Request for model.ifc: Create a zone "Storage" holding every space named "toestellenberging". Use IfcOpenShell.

First a look at what the model holds.

```python
import ifcopenshell

model = ifcopenshell.open("model.ifc")
print(model.schema)
seen = {}
for space in model.by_type("IfcSpace"):
    seen[space.LongName] = seen.get(space.LongName, 0) + 1
for name, count in sorted(seen.items(), key=str):
    print(count, "x", name)
print("zones:", [z.Name for z in model.by_type("IfcZone")][:20])
```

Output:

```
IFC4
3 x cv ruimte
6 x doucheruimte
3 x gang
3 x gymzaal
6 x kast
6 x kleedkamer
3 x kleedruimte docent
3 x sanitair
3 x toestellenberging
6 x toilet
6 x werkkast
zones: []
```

```python
import ifcopenshell
import ifcopenshell.api.group
import ifcopenshell.api.root

model = ifcopenshell.open("model.ifc")

names = {"toestellenberging"}
spaces = [s for s in model.by_type("IfcSpace") if s.LongName in names]

zone = ifcopenshell.api.root.create_entity(model, ifc_class="IfcZone", name="Storage")
ifcopenshell.api.group.assign_group(model, products=spaces, group=zone)
print(len(spaces), "spaces in", zone.Name)

model.write("model_v2.ifc")
```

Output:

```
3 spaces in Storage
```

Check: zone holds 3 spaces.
